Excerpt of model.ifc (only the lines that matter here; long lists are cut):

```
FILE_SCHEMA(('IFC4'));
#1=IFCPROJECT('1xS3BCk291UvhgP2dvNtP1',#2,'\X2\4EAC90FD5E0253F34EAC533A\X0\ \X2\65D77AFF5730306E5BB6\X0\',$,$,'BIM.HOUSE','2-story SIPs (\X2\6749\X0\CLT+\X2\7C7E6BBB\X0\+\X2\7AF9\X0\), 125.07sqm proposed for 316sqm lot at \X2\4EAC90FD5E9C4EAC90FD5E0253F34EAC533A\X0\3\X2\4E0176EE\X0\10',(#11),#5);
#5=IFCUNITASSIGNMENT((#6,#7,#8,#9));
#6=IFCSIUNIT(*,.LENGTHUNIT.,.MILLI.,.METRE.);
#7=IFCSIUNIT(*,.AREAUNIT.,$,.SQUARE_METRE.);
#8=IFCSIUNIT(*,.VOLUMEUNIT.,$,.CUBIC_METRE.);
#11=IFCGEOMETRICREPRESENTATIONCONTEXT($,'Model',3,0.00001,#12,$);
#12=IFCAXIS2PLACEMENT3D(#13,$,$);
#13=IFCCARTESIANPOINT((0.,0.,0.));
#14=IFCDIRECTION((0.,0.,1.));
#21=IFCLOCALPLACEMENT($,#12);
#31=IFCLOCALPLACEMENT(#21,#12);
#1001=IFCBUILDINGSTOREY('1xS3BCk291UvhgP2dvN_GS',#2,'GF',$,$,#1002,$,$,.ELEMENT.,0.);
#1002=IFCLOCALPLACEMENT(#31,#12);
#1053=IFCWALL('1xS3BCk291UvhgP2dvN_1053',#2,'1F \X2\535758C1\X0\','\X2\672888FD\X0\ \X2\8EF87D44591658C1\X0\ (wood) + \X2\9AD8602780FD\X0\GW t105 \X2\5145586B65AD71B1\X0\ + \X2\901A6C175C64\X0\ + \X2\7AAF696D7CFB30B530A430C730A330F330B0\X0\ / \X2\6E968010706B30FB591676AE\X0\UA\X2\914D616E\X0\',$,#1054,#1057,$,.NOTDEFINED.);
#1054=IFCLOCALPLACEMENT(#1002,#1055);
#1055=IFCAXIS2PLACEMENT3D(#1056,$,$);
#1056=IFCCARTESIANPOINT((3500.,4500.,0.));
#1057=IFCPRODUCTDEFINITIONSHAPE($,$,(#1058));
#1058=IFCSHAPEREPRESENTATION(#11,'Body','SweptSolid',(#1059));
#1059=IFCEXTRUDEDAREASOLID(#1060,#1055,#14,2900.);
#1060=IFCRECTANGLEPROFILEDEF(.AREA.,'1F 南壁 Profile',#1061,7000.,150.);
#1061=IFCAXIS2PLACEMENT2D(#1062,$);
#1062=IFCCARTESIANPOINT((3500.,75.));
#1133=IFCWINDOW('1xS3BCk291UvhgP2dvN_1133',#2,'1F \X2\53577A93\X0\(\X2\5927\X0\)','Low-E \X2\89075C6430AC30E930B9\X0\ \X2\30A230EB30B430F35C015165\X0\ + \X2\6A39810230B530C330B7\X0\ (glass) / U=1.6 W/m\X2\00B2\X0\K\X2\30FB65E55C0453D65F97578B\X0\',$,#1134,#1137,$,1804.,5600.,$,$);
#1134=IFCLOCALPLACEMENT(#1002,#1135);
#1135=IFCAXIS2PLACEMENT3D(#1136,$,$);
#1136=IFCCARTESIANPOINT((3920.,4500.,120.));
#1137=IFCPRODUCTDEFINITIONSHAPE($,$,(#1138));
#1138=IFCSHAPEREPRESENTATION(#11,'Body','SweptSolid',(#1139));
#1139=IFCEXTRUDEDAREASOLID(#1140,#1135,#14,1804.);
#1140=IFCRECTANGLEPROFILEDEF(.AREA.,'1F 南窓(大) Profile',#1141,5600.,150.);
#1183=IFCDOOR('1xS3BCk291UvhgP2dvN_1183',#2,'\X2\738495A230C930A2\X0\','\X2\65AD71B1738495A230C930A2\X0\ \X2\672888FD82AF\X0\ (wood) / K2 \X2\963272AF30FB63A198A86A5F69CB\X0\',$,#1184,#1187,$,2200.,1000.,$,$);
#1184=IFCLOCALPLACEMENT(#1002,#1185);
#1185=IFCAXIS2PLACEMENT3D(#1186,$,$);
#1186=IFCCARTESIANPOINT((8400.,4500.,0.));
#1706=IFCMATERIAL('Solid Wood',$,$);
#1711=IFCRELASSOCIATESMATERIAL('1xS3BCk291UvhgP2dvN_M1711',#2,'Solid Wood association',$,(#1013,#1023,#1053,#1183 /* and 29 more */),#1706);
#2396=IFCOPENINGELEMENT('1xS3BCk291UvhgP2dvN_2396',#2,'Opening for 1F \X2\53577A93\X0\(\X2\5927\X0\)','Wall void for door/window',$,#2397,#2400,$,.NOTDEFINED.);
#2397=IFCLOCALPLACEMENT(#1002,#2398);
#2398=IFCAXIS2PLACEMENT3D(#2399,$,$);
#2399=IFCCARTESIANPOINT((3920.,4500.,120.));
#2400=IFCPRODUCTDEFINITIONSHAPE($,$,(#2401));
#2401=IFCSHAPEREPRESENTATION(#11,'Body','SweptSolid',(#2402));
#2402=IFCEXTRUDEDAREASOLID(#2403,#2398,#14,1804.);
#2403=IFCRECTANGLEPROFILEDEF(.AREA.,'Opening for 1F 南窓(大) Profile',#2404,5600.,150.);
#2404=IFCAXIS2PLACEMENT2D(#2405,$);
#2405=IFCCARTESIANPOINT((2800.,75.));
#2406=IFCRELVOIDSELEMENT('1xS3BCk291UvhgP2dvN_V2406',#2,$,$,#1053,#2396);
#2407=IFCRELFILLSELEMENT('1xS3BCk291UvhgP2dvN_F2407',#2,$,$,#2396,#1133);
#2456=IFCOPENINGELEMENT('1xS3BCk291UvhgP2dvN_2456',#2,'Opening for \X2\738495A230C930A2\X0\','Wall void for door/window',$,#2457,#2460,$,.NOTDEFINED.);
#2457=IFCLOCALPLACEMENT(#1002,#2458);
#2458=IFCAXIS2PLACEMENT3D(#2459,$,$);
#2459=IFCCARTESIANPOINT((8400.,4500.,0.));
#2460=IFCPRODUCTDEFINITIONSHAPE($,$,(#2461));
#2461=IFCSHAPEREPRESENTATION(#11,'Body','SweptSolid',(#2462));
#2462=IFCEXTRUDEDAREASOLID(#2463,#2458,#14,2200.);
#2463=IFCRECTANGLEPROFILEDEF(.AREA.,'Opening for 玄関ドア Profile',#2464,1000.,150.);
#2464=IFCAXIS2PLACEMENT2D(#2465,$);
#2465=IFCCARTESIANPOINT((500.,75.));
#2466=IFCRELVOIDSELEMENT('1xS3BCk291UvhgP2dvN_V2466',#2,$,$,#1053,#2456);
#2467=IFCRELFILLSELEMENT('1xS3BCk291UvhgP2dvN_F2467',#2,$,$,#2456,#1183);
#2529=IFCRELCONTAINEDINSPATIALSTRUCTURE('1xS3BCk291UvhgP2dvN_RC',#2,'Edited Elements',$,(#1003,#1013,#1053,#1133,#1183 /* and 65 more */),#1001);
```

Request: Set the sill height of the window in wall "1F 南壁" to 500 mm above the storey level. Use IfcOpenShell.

```python
import numpy as np
import ifcopenshell
import ifcopenshell.api.geometry
import ifcopenshell.geom
import ifcopenshell.util.element
import ifcopenshell.util.placement
import ifcopenshell.util.shape
import ifcopenshell.util.unit

model = ifcopenshell.open("model.ifc")
unit_scale = ifcopenshell.util.unit.calculate_unit_scale(model)

window = model.by_guid("1xS3BCk291UvhgP2dvN_1133")
opening = window.FillsVoids[0].RelatingOpeningElement
storey = ifcopenshell.util.element.get_container(window, ifc_class="IfcBuildingStorey")
level = ifcopenshell.util.placement.get_local_placement(storey.ObjectPlacement)[2, 3]

# The opening's origin need not be at the sill, so measure its lowest point.
shape = ifcopenshell.geom.create_shape(ifcopenshell.geom.settings(), opening)
bottom = ifcopenshell.util.shape.get_shape_bottom_elevation(shape, shape.geometry) / unit_scale
dz = level + 0.5 / unit_scale - bottom

shift = np.array([0.0, 0.0, dz])
# The window is not placed relative to its opening, so move both.
for product in (opening, window):
    matrix = ifcopenshell.util.placement.get_local_placement(product.ObjectPlacement)
    matrix[:3, 3] += shift
    ifcopenshell.api.geometry.edit_object_placement(model, product=product, matrix=matrix, is_si=False)

print(f"moved by {dz * unit_scale:+.3f} m")

model.write("model_v2.ifc")
```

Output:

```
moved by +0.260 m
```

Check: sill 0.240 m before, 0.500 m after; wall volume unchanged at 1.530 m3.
